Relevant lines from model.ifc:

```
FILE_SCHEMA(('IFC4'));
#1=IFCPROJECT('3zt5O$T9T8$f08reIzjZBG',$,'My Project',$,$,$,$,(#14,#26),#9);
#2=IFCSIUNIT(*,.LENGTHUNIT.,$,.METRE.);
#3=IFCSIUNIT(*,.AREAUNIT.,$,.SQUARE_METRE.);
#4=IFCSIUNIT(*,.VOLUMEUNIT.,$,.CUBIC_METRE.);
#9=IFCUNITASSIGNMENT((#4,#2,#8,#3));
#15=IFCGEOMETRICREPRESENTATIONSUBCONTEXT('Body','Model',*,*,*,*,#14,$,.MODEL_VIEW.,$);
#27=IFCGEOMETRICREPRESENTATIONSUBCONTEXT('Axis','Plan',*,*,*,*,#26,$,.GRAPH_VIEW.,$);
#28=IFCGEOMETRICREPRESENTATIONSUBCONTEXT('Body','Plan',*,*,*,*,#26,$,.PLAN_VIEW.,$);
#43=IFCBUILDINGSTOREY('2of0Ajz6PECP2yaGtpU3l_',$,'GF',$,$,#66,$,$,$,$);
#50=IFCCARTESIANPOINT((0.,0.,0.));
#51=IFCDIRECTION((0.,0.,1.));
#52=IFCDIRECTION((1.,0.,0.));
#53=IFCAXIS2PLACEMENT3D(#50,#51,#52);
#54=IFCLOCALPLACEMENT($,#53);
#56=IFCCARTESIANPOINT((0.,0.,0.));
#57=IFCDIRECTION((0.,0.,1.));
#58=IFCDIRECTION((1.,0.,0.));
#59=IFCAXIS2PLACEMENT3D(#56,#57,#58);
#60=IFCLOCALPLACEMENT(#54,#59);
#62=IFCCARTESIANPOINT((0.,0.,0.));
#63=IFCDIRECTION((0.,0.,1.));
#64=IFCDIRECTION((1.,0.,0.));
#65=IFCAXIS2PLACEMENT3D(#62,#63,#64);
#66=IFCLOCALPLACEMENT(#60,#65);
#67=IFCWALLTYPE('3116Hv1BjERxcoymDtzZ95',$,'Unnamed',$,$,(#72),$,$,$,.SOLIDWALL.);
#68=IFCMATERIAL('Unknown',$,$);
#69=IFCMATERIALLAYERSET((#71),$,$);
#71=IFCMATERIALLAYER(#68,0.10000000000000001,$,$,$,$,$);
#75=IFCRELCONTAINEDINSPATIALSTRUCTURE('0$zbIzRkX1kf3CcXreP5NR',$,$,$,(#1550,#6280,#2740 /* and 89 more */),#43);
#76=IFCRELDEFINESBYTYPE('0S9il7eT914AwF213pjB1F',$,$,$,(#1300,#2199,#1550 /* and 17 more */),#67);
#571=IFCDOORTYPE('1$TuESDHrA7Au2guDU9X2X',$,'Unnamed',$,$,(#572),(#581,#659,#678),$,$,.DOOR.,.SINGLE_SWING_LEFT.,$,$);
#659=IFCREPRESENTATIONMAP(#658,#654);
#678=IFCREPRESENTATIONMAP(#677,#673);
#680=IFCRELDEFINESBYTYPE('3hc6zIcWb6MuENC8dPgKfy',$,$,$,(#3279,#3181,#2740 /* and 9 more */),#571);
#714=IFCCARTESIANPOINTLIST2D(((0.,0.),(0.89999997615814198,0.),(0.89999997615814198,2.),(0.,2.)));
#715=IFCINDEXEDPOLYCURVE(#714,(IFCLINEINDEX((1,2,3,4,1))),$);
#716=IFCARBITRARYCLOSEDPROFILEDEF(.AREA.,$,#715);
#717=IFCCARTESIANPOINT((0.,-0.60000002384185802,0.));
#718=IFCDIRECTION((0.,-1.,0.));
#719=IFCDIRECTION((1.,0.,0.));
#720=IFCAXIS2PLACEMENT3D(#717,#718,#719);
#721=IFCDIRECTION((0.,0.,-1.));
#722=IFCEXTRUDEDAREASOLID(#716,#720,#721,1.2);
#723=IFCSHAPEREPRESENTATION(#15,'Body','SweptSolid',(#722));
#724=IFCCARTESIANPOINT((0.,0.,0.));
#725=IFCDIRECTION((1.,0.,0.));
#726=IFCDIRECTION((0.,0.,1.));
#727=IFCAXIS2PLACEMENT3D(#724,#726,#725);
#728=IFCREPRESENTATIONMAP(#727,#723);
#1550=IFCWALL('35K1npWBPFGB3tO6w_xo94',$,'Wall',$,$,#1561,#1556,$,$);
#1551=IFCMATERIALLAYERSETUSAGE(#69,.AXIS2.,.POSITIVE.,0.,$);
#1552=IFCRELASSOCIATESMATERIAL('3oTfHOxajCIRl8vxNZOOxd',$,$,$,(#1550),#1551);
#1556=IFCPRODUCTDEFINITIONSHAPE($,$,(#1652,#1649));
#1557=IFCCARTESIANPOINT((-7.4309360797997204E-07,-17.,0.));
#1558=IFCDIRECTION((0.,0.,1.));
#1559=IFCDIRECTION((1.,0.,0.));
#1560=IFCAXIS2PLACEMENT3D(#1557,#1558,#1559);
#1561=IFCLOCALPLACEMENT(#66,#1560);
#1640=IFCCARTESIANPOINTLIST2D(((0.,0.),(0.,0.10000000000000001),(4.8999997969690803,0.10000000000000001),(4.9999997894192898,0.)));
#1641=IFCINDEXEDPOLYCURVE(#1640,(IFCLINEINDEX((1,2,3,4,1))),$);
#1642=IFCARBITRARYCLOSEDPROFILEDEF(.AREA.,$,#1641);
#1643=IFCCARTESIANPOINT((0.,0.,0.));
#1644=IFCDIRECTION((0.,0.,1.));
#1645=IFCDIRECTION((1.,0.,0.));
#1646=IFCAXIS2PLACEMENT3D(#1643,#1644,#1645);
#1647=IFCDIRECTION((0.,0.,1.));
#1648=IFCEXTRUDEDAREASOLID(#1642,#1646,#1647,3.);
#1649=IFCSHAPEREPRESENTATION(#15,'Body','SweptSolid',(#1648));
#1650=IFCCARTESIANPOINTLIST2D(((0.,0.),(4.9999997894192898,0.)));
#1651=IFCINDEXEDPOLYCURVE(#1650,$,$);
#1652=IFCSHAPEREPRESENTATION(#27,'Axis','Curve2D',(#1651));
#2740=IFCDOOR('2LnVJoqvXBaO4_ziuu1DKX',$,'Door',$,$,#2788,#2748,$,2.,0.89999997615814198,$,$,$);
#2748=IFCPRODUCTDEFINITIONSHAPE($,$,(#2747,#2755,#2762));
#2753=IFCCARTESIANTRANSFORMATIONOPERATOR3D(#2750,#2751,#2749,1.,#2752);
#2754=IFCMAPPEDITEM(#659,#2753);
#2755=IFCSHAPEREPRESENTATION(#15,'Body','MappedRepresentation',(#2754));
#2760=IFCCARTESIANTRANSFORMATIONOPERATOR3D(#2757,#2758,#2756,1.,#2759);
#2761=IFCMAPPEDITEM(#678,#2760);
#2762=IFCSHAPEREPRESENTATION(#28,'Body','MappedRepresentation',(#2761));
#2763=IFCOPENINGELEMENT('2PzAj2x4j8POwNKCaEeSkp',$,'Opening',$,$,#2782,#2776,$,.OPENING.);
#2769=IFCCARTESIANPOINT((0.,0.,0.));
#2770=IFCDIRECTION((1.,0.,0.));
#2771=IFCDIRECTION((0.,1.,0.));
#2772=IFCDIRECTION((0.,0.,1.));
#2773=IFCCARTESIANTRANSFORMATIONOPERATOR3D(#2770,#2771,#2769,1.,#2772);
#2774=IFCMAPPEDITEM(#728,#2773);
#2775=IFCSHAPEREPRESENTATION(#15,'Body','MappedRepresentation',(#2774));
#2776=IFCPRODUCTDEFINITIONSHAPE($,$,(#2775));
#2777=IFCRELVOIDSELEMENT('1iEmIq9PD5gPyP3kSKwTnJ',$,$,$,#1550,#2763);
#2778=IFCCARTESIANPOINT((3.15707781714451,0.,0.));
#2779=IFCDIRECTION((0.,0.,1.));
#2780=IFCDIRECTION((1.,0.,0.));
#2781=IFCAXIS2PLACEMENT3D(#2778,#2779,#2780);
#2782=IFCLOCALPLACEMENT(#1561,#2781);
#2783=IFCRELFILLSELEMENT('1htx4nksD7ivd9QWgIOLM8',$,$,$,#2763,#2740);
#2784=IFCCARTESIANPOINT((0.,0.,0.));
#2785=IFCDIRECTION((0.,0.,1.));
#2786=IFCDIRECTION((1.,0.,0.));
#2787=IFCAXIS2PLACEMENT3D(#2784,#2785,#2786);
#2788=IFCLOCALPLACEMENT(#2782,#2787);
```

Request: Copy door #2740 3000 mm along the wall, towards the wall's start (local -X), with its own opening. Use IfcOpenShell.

```python
import ifcopenshell
import ifcopenshell.api.feature
import ifcopenshell.api.geometry
import ifcopenshell.api.root
import ifcopenshell.geom
import ifcopenshell.util.element
import ifcopenshell.util.placement
import ifcopenshell.util.shape
import ifcopenshell.util.unit

model = ifcopenshell.open("model.ifc")
unit_scale = ifcopenshell.util.unit.calculate_unit_scale(model)
settings = ifcopenshell.geom.settings()


def volume(element):
    """Net volume in cubic metres, openings subtracted."""
    shape = ifcopenshell.geom.create_shape(settings, element)
    return ifcopenshell.util.shape.get_volume(shape.geometry)


door = model.by_guid("2LnVJoqvXBaO4_ziuu1DKX")
opening = door.FillsVoids[0].RelatingOpeningElement
wall = opening.VoidsElements[0].RelatingBuildingElement
before = volume(wall)
shift = ifcopenshell.util.placement.get_local_placement(wall.ObjectPlacement)[:3, 0] * -3 / unit_scale

# copy_class copies the void relationship, type, container and properties, but no geometry.
new_opening = ifcopenshell.api.root.copy_class(model, product=opening)
new_opening.Representation = ifcopenshell.util.element.copy_deep(
    model, opening.Representation, exclude=["IfcGeometricRepresentationContext", "IfcRepresentationMap"]
)
new_door = ifcopenshell.api.root.copy_class(model, product=door)
new_door.Representation = ifcopenshell.util.element.copy_deep(
    model, door.Representation, exclude=["IfcGeometricRepresentationContext", "IfcRepresentationMap"]
)
ifcopenshell.api.feature.add_filling(model, opening=new_opening, element=new_door)

for old, new in ((opening, new_opening), (door, new_door)):
    matrix = ifcopenshell.util.placement.get_local_placement(old.ObjectPlacement)
    matrix[:3, 3] += shift
    ifcopenshell.api.geometry.edit_object_placement(model, product=new, matrix=matrix, is_si=False)

after = volume(wall)

print(f"wall volume {before:.3f} -> {after:.3f} m3")

model.write("model_v2.ifc")
```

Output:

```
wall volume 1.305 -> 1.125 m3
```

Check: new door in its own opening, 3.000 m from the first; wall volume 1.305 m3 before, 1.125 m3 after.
